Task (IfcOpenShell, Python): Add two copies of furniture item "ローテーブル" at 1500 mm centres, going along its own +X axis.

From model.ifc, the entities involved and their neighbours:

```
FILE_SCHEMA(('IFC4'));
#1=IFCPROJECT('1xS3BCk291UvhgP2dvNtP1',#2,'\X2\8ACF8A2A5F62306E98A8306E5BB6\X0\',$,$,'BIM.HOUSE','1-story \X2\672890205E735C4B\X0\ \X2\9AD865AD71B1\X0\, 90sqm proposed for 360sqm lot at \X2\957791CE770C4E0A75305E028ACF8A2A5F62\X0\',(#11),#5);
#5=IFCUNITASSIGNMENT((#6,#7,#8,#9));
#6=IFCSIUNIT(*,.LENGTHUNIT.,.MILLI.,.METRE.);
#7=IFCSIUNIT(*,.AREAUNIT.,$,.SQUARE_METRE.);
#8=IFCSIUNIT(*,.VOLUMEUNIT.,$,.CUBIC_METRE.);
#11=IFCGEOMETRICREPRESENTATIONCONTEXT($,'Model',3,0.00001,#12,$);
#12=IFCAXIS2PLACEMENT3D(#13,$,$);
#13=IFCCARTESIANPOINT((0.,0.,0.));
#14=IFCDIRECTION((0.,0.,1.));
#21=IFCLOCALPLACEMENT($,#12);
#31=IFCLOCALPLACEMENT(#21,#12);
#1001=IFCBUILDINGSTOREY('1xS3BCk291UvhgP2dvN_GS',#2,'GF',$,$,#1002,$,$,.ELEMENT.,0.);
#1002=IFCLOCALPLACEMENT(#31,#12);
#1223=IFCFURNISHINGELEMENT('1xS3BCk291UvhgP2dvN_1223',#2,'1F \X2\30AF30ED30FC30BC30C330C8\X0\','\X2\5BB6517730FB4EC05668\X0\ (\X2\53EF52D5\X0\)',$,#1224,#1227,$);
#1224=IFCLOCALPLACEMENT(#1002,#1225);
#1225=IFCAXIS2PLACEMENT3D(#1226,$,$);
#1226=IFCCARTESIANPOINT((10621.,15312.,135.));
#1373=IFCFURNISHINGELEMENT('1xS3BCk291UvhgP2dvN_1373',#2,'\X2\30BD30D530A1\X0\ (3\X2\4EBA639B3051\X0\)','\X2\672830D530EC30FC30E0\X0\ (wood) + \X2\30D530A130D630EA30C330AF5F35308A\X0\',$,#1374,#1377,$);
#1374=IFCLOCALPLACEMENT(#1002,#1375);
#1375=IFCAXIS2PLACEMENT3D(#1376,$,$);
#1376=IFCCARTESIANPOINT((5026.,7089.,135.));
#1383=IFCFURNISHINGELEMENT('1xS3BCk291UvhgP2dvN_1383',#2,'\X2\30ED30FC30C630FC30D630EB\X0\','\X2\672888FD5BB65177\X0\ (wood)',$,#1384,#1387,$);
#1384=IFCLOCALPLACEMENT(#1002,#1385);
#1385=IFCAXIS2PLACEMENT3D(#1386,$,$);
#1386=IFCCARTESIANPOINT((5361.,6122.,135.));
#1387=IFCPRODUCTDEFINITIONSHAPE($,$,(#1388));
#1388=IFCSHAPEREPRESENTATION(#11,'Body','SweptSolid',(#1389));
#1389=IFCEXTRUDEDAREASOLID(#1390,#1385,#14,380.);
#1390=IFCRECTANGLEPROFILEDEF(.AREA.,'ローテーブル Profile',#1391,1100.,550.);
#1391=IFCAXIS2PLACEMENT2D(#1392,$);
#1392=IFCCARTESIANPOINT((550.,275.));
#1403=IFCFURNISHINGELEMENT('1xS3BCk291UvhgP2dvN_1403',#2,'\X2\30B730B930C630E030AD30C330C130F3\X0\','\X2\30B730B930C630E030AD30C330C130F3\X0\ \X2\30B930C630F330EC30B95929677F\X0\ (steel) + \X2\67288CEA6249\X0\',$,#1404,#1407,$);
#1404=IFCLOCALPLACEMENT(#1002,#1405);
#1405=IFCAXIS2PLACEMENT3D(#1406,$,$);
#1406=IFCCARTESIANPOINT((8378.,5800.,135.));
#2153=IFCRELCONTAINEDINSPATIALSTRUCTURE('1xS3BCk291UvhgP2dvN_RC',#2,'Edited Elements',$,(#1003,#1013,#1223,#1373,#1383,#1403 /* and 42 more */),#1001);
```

```python
import ifcopenshell
import ifcopenshell.api.geometry
import ifcopenshell.api.root
import ifcopenshell.util.element
import ifcopenshell.util.placement
import ifcopenshell.util.unit

model = ifcopenshell.open("model.ifc")
unit_scale = ifcopenshell.util.unit.calculate_unit_scale(model)


def reuse_history(source, copy):
    """copy_class also copies each property set's owner history, people and application; keep the originals."""
    for rel in copy.IsDefinedBy:
        if rel.is_a("IfcRelDefinesByProperties") and (history := rel.RelatingPropertyDefinition.OwnerHistory):
            rel.RelatingPropertyDefinition.OwnerHistory = source.OwnerHistory
            ifcopenshell.util.element.remove_deep2(model, history)


source = model.by_guid("1xS3BCk291UvhgP2dvN_1383")
base = ifcopenshell.util.placement.get_local_placement(source.ObjectPlacement)
step = base[:3, 0] * 1.5 / unit_scale

for i in range(1, 3):
    copy = ifcopenshell.api.root.copy_class(model, product=source)
    copy.Representation = ifcopenshell.util.element.copy_deep(
        model, source.Representation, exclude=["IfcGeometricRepresentationContext", "IfcRepresentationMap"]
    )
    reuse_history(source, copy)
    matrix = base.copy()
    matrix[:3, 3] += i * step
    print("added at", matrix[:3, 3].round(3) + 0.0)
    ifcopenshell.api.geometry.edit_object_placement(model, product=copy, matrix=matrix, is_si=False)

model.write("model_rev.ifc")
```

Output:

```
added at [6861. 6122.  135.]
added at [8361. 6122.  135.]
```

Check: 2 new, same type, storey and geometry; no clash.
